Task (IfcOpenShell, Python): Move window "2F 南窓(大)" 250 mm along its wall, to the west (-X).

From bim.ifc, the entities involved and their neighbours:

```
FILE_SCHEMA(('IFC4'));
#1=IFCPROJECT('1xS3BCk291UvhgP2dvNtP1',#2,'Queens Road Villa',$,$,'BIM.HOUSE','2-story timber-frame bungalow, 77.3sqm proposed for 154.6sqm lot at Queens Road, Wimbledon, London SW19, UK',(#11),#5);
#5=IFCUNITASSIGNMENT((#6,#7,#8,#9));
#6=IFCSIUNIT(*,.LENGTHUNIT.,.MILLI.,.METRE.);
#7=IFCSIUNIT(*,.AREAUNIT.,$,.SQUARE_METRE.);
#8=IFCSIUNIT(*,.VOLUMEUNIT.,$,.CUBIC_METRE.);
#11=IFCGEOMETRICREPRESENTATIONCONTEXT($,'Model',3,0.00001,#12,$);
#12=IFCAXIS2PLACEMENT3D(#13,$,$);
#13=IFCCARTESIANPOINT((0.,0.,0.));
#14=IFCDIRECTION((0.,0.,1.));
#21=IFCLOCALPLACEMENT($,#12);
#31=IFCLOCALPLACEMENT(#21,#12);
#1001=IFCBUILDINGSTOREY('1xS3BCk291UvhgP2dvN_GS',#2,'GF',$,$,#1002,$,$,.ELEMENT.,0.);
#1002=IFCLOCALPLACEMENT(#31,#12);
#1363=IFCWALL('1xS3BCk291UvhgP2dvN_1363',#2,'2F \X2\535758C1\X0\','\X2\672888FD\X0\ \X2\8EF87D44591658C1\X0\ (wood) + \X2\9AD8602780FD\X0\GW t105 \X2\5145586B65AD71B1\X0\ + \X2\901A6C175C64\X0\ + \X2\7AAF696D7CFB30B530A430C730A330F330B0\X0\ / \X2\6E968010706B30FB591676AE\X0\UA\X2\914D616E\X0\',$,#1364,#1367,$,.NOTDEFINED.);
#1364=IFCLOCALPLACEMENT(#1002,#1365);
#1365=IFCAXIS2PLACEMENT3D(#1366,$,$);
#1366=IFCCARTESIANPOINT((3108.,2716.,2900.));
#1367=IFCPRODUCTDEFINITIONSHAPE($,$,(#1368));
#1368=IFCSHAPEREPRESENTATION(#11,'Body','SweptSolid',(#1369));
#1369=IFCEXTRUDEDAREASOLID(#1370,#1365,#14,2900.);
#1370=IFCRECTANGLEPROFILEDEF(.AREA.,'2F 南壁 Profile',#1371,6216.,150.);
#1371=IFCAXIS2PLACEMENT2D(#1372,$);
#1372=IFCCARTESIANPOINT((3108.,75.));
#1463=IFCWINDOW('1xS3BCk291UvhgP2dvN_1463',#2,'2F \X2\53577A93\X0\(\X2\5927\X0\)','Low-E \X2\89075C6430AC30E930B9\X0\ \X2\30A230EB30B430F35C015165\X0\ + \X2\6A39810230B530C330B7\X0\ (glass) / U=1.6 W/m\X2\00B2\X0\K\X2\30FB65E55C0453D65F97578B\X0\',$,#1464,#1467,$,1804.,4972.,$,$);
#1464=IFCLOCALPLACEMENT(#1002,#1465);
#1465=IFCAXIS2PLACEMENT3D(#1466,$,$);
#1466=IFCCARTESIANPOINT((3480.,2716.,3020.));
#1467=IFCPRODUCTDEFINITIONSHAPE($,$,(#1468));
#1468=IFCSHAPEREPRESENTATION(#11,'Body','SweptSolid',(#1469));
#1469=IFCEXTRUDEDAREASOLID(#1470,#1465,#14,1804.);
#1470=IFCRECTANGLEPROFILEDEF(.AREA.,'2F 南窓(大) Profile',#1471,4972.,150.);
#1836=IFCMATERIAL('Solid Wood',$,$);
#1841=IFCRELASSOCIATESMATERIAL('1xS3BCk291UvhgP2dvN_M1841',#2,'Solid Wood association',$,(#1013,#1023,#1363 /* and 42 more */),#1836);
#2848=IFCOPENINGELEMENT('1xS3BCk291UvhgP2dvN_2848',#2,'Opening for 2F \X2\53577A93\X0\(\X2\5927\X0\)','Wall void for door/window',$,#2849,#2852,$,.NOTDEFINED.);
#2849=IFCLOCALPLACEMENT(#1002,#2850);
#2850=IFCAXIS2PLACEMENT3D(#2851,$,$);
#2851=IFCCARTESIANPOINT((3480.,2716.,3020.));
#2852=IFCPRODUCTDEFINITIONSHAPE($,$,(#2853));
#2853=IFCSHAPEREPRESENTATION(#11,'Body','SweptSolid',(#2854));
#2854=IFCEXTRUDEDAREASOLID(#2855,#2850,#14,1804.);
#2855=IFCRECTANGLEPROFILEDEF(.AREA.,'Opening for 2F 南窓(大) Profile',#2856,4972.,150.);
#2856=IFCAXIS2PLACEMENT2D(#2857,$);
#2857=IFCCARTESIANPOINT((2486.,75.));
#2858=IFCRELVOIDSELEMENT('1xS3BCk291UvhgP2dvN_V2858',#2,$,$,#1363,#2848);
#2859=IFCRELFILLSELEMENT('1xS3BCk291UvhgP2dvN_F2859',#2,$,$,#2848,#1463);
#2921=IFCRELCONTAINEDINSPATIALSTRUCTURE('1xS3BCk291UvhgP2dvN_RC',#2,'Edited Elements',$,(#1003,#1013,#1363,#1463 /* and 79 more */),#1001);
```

```python
import ifcopenshell
import ifcopenshell.api.geometry
import ifcopenshell.util.placement
import ifcopenshell.util.unit

model = ifcopenshell.open("bim.ifc")
unit_scale = ifcopenshell.util.unit.calculate_unit_scale(model)

window = model.by_guid("1xS3BCk291UvhgP2dvN_1463")
opening = window.FillsVoids[0].RelatingOpeningElement
wall = opening.VoidsElements[0].RelatingBuildingElement

wall_matrix = ifcopenshell.util.placement.get_local_placement(wall.ObjectPlacement)
shift = wall_matrix[:3, 0] * -0.25 / unit_scale
before = ifcopenshell.util.placement.get_local_placement(window.ObjectPlacement)[:3, 3].copy()

# The window is not placed relative to its opening, so move both.
for product in (opening, window):
    matrix = ifcopenshell.util.placement.get_local_placement(product.ObjectPlacement)
    matrix[:3, 3] += shift
    ifcopenshell.api.geometry.edit_object_placement(model, product=product, matrix=matrix, is_si=False)

after = ifcopenshell.util.placement.get_local_placement(window.ObjectPlacement)[:3, 3]
print("window moved by", (after - before).round(3) + 0.0)

model.write("bim-out.ifc")
```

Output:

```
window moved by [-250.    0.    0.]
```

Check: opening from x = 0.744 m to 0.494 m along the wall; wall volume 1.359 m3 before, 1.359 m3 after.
